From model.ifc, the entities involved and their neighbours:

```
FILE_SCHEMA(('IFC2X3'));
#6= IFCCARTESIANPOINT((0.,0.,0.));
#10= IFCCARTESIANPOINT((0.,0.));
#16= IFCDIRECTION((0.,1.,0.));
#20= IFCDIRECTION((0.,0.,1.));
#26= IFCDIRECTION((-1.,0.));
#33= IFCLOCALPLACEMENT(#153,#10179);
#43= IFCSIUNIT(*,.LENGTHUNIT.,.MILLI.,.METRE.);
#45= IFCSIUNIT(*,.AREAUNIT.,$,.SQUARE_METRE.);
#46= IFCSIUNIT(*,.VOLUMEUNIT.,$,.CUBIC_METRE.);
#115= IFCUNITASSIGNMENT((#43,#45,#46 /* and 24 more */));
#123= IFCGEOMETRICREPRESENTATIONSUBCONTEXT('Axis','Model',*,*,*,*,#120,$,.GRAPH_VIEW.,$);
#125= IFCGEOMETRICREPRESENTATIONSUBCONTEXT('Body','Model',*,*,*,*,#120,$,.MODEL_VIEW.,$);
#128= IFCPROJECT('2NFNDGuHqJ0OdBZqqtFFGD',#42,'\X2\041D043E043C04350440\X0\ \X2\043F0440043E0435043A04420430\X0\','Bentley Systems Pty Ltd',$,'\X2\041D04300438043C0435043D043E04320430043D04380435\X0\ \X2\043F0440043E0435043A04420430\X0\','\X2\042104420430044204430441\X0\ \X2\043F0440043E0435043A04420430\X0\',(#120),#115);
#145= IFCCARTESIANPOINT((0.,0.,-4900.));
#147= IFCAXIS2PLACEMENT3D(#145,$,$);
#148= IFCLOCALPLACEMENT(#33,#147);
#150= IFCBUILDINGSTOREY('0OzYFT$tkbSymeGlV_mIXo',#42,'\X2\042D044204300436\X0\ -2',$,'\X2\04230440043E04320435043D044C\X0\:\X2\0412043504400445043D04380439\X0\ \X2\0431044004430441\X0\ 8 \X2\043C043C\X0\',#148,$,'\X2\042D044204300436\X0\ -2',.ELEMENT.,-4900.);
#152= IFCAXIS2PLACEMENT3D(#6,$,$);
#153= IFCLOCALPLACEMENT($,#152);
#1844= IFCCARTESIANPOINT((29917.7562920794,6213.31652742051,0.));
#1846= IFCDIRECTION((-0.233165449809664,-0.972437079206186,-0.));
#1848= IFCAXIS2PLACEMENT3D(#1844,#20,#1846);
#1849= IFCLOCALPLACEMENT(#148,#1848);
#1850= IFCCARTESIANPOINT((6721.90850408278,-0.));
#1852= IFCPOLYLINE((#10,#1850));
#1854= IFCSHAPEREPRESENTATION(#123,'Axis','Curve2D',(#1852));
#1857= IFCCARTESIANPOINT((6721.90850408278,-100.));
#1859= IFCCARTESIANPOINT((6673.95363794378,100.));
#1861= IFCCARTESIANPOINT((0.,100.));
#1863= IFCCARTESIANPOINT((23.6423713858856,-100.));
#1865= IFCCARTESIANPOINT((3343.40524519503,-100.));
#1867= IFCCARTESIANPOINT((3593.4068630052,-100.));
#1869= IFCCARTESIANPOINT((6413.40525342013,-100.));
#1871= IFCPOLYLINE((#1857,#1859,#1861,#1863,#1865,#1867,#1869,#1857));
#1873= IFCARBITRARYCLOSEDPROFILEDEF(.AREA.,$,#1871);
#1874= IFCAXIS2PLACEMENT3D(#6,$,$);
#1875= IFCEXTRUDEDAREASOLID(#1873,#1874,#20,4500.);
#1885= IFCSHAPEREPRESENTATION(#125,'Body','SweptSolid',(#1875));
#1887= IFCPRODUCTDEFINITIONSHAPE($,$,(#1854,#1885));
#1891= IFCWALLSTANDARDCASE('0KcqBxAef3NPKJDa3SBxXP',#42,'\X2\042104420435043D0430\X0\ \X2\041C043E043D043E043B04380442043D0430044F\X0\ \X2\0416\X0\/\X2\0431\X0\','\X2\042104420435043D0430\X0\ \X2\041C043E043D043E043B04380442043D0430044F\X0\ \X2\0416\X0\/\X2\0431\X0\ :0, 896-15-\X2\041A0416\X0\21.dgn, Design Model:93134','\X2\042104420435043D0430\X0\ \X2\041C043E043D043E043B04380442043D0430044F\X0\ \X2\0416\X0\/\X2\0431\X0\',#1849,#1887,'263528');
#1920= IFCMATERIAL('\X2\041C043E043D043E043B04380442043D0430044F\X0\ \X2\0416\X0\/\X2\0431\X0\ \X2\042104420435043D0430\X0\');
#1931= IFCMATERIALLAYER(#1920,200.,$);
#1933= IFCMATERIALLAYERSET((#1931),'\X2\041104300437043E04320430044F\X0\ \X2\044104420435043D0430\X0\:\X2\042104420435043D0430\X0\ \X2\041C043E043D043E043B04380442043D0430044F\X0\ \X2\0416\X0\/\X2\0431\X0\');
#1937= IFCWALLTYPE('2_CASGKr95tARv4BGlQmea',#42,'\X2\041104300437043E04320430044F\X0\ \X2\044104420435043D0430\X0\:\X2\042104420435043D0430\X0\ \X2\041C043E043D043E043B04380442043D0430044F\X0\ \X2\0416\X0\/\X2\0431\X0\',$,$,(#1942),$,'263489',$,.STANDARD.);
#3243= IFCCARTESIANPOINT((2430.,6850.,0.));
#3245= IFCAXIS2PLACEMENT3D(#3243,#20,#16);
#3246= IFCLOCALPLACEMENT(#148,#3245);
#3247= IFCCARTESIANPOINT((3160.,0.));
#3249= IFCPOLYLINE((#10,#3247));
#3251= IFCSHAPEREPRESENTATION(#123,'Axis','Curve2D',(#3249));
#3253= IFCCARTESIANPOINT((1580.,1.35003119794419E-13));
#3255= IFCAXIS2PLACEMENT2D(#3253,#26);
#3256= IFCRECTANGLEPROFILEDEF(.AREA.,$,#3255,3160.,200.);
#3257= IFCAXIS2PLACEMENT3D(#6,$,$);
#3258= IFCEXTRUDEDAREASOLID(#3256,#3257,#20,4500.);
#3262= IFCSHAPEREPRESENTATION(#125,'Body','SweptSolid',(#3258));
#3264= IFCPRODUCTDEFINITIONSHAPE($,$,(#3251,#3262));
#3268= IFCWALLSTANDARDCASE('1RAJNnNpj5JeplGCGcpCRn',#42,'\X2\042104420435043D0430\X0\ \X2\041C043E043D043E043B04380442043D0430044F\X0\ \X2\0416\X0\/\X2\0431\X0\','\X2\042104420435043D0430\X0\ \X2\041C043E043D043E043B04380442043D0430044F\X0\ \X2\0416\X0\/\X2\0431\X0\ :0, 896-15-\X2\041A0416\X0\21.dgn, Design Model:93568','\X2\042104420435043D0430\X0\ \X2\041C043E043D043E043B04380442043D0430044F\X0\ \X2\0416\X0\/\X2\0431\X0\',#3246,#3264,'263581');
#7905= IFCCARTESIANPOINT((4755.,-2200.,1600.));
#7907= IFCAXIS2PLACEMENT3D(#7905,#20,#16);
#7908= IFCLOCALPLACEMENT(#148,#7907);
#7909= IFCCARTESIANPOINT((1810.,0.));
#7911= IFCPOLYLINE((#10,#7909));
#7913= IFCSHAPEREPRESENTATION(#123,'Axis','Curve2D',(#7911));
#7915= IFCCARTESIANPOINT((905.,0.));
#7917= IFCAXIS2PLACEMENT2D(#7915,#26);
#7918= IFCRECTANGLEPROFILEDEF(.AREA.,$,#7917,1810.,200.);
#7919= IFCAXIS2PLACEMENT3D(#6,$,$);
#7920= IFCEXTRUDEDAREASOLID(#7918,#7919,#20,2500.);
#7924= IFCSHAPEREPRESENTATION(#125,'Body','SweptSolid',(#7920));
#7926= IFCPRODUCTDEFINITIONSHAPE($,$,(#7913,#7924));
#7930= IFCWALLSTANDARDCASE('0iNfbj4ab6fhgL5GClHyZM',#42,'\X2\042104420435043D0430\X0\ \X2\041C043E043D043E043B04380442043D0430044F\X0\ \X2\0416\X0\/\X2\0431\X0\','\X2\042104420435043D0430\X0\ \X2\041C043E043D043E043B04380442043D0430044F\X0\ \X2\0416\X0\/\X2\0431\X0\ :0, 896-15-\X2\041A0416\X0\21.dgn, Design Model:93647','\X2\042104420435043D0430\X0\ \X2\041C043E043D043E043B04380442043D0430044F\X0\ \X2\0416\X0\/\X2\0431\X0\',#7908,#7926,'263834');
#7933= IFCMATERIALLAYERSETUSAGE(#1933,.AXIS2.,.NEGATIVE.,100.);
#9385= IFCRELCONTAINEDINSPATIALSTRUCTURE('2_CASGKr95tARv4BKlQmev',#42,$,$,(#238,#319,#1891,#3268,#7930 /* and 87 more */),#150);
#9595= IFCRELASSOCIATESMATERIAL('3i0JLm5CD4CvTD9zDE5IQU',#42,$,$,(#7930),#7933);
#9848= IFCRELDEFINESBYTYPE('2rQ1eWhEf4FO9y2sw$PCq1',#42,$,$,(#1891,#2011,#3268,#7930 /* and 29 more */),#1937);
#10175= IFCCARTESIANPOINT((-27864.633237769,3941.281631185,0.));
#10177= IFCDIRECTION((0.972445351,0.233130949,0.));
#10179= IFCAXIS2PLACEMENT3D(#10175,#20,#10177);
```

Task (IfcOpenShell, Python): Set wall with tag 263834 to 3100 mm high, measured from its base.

```python
import ifcopenshell
import ifcopenshell.geom
import ifcopenshell.util.representation
import ifcopenshell.util.shape

model = ifcopenshell.open("model.ifc")
settings = ifcopenshell.geom.settings()


def volume(element):
    """Net volume in cubic metres, openings subtracted."""
    shape = ifcopenshell.geom.create_shape(settings, element)
    return ifcopenshell.util.shape.get_volume(shape.geometry)


wall = model.by_id(7930)
before = volume(wall)

body = ifcopenshell.util.representation.get_representation(wall, "Model", "Body")
solid = body.Items[0]
old_height = solid.Depth
solid.Depth = 3100.0
after = volume(wall)

print(f"height {old_height:g} -> {solid.Depth:g}, volume {before:.3f} -> {after:.3f} m3")

model.write("model_v2.ifc")
```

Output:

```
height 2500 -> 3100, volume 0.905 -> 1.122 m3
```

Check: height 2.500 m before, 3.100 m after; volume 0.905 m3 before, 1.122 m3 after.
